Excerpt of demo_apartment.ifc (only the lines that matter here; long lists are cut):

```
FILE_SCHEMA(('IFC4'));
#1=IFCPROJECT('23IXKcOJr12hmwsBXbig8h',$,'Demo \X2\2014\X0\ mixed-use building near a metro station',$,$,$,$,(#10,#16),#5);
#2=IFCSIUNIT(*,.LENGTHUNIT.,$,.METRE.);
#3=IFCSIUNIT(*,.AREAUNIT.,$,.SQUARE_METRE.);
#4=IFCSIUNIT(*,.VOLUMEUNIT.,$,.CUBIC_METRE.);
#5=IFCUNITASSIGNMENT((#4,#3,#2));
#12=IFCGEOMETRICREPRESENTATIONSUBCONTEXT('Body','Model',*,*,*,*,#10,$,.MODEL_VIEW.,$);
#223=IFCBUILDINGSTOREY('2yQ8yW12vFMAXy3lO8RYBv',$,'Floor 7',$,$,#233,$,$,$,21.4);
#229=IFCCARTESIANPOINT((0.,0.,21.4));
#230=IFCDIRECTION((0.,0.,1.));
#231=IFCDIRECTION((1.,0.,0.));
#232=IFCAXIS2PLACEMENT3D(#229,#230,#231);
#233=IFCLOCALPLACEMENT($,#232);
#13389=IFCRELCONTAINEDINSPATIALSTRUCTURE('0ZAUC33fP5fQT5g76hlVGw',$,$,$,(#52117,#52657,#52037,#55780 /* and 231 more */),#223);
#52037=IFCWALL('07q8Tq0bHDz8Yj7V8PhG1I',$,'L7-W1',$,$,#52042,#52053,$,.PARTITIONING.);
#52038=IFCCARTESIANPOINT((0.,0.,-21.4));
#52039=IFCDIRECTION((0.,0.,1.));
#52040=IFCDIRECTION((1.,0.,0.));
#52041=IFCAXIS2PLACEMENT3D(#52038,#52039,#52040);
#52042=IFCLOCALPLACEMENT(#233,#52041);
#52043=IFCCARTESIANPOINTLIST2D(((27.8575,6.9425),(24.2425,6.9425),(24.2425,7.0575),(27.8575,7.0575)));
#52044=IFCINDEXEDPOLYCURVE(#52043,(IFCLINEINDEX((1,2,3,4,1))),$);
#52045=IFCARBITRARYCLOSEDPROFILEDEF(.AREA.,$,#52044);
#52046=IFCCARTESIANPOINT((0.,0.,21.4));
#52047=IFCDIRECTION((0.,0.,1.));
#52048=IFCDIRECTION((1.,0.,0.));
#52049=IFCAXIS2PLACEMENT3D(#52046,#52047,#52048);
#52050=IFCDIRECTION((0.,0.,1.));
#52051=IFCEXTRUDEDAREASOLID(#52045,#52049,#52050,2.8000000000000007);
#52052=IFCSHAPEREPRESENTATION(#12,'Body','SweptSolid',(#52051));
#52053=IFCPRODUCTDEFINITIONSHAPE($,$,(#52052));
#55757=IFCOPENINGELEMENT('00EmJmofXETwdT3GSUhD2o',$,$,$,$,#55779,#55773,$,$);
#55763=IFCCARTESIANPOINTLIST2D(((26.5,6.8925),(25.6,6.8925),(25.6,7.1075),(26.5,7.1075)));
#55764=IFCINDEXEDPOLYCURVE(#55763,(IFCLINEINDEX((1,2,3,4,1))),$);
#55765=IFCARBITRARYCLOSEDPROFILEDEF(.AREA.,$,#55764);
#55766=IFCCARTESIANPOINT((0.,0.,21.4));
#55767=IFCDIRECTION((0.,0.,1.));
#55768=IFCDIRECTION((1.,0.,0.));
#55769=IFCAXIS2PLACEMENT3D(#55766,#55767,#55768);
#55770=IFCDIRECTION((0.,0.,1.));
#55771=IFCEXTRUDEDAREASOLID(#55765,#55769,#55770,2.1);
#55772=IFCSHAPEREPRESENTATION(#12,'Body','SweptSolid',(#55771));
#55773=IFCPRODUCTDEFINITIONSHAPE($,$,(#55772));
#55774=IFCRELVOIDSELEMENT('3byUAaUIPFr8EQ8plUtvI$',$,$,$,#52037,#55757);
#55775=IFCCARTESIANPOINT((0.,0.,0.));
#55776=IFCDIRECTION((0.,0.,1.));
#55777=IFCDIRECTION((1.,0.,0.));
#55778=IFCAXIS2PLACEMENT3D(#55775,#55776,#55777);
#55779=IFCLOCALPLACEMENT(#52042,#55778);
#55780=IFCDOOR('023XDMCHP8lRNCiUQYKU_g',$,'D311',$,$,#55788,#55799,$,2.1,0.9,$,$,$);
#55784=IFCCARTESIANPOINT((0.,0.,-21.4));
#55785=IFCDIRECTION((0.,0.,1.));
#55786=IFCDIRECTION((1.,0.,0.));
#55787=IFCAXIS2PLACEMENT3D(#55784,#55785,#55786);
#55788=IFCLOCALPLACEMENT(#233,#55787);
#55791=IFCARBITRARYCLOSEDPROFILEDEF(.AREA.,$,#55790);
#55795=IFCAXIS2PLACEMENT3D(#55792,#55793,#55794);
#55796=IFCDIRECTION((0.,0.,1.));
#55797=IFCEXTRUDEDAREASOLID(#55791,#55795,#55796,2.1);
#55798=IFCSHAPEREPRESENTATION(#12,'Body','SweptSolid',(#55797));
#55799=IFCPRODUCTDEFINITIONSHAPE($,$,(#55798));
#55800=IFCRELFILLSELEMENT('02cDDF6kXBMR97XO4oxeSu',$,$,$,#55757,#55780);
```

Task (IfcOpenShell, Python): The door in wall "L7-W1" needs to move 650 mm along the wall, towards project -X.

```python
import ifcopenshell
import ifcopenshell.api.geometry
import ifcopenshell.util.placement

model = ifcopenshell.open("demo_apartment.ifc")

door = model.by_guid("023XDMCHP8lRNCiUQYKU_g")
opening = door.FillsVoids[0].RelatingOpeningElement
wall = opening.VoidsElements[0].RelatingBuildingElement

wall_matrix = ifcopenshell.util.placement.get_local_placement(wall.ObjectPlacement)
shift = wall_matrix[:3, 0] * -0.65
before = ifcopenshell.util.placement.get_local_placement(door.ObjectPlacement)[:3, 3].copy()

# The door is not placed relative to its opening, so move both.
for product in (opening, door):
    matrix = ifcopenshell.util.placement.get_local_placement(product.ObjectPlacement)
    matrix[:3, 3] += shift
    ifcopenshell.api.geometry.edit_object_placement(model, product=product, matrix=matrix, is_si=False)

after = ifcopenshell.util.placement.get_local_placement(door.ObjectPlacement)[:3, 3]
print("door moved by", (after - before).round(3) + 0.0)

model.write("demo_apartment_edited.ifc")
```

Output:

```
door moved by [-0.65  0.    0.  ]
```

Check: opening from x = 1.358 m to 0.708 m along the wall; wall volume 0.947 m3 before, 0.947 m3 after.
